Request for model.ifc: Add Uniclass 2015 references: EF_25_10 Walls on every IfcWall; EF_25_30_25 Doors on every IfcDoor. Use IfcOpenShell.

First a look at what the model holds.

```python
import ifcopenshell

model = ifcopenshell.open("model.ifc")
print(model.schema)
print("classifications:", [c.Name for c in model.by_type("IfcClassification")])
for ifc_class in ("IfcDoor", "IfcRoof", "IfcStair", "IfcWall", "IfcWindow"):
    print(ifc_class, len(model.by_type(ifc_class)))
```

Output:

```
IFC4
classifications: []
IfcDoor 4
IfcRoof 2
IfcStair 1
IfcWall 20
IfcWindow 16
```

```python
import ifcopenshell
import ifcopenshell.api.classification

model = ifcopenshell.open("model.ifc")

system = ifcopenshell.api.classification.add_classification(model, classification="Uniclass 2015")

codes = {
    "IfcWall": ("EF_25_10", "Walls"),
    "IfcDoor": ("EF_25_30_25", "Doors"),
}
for ifc_class, (code, name) in codes.items():
    products = model.by_type(ifc_class)
    ifcopenshell.api.classification.add_reference(
        model, products=products, classification=system, identification=code, name=name
    )
    print(code, len(products))

model.write("model-out.ifc")
```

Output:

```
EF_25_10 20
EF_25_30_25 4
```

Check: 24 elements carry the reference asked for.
